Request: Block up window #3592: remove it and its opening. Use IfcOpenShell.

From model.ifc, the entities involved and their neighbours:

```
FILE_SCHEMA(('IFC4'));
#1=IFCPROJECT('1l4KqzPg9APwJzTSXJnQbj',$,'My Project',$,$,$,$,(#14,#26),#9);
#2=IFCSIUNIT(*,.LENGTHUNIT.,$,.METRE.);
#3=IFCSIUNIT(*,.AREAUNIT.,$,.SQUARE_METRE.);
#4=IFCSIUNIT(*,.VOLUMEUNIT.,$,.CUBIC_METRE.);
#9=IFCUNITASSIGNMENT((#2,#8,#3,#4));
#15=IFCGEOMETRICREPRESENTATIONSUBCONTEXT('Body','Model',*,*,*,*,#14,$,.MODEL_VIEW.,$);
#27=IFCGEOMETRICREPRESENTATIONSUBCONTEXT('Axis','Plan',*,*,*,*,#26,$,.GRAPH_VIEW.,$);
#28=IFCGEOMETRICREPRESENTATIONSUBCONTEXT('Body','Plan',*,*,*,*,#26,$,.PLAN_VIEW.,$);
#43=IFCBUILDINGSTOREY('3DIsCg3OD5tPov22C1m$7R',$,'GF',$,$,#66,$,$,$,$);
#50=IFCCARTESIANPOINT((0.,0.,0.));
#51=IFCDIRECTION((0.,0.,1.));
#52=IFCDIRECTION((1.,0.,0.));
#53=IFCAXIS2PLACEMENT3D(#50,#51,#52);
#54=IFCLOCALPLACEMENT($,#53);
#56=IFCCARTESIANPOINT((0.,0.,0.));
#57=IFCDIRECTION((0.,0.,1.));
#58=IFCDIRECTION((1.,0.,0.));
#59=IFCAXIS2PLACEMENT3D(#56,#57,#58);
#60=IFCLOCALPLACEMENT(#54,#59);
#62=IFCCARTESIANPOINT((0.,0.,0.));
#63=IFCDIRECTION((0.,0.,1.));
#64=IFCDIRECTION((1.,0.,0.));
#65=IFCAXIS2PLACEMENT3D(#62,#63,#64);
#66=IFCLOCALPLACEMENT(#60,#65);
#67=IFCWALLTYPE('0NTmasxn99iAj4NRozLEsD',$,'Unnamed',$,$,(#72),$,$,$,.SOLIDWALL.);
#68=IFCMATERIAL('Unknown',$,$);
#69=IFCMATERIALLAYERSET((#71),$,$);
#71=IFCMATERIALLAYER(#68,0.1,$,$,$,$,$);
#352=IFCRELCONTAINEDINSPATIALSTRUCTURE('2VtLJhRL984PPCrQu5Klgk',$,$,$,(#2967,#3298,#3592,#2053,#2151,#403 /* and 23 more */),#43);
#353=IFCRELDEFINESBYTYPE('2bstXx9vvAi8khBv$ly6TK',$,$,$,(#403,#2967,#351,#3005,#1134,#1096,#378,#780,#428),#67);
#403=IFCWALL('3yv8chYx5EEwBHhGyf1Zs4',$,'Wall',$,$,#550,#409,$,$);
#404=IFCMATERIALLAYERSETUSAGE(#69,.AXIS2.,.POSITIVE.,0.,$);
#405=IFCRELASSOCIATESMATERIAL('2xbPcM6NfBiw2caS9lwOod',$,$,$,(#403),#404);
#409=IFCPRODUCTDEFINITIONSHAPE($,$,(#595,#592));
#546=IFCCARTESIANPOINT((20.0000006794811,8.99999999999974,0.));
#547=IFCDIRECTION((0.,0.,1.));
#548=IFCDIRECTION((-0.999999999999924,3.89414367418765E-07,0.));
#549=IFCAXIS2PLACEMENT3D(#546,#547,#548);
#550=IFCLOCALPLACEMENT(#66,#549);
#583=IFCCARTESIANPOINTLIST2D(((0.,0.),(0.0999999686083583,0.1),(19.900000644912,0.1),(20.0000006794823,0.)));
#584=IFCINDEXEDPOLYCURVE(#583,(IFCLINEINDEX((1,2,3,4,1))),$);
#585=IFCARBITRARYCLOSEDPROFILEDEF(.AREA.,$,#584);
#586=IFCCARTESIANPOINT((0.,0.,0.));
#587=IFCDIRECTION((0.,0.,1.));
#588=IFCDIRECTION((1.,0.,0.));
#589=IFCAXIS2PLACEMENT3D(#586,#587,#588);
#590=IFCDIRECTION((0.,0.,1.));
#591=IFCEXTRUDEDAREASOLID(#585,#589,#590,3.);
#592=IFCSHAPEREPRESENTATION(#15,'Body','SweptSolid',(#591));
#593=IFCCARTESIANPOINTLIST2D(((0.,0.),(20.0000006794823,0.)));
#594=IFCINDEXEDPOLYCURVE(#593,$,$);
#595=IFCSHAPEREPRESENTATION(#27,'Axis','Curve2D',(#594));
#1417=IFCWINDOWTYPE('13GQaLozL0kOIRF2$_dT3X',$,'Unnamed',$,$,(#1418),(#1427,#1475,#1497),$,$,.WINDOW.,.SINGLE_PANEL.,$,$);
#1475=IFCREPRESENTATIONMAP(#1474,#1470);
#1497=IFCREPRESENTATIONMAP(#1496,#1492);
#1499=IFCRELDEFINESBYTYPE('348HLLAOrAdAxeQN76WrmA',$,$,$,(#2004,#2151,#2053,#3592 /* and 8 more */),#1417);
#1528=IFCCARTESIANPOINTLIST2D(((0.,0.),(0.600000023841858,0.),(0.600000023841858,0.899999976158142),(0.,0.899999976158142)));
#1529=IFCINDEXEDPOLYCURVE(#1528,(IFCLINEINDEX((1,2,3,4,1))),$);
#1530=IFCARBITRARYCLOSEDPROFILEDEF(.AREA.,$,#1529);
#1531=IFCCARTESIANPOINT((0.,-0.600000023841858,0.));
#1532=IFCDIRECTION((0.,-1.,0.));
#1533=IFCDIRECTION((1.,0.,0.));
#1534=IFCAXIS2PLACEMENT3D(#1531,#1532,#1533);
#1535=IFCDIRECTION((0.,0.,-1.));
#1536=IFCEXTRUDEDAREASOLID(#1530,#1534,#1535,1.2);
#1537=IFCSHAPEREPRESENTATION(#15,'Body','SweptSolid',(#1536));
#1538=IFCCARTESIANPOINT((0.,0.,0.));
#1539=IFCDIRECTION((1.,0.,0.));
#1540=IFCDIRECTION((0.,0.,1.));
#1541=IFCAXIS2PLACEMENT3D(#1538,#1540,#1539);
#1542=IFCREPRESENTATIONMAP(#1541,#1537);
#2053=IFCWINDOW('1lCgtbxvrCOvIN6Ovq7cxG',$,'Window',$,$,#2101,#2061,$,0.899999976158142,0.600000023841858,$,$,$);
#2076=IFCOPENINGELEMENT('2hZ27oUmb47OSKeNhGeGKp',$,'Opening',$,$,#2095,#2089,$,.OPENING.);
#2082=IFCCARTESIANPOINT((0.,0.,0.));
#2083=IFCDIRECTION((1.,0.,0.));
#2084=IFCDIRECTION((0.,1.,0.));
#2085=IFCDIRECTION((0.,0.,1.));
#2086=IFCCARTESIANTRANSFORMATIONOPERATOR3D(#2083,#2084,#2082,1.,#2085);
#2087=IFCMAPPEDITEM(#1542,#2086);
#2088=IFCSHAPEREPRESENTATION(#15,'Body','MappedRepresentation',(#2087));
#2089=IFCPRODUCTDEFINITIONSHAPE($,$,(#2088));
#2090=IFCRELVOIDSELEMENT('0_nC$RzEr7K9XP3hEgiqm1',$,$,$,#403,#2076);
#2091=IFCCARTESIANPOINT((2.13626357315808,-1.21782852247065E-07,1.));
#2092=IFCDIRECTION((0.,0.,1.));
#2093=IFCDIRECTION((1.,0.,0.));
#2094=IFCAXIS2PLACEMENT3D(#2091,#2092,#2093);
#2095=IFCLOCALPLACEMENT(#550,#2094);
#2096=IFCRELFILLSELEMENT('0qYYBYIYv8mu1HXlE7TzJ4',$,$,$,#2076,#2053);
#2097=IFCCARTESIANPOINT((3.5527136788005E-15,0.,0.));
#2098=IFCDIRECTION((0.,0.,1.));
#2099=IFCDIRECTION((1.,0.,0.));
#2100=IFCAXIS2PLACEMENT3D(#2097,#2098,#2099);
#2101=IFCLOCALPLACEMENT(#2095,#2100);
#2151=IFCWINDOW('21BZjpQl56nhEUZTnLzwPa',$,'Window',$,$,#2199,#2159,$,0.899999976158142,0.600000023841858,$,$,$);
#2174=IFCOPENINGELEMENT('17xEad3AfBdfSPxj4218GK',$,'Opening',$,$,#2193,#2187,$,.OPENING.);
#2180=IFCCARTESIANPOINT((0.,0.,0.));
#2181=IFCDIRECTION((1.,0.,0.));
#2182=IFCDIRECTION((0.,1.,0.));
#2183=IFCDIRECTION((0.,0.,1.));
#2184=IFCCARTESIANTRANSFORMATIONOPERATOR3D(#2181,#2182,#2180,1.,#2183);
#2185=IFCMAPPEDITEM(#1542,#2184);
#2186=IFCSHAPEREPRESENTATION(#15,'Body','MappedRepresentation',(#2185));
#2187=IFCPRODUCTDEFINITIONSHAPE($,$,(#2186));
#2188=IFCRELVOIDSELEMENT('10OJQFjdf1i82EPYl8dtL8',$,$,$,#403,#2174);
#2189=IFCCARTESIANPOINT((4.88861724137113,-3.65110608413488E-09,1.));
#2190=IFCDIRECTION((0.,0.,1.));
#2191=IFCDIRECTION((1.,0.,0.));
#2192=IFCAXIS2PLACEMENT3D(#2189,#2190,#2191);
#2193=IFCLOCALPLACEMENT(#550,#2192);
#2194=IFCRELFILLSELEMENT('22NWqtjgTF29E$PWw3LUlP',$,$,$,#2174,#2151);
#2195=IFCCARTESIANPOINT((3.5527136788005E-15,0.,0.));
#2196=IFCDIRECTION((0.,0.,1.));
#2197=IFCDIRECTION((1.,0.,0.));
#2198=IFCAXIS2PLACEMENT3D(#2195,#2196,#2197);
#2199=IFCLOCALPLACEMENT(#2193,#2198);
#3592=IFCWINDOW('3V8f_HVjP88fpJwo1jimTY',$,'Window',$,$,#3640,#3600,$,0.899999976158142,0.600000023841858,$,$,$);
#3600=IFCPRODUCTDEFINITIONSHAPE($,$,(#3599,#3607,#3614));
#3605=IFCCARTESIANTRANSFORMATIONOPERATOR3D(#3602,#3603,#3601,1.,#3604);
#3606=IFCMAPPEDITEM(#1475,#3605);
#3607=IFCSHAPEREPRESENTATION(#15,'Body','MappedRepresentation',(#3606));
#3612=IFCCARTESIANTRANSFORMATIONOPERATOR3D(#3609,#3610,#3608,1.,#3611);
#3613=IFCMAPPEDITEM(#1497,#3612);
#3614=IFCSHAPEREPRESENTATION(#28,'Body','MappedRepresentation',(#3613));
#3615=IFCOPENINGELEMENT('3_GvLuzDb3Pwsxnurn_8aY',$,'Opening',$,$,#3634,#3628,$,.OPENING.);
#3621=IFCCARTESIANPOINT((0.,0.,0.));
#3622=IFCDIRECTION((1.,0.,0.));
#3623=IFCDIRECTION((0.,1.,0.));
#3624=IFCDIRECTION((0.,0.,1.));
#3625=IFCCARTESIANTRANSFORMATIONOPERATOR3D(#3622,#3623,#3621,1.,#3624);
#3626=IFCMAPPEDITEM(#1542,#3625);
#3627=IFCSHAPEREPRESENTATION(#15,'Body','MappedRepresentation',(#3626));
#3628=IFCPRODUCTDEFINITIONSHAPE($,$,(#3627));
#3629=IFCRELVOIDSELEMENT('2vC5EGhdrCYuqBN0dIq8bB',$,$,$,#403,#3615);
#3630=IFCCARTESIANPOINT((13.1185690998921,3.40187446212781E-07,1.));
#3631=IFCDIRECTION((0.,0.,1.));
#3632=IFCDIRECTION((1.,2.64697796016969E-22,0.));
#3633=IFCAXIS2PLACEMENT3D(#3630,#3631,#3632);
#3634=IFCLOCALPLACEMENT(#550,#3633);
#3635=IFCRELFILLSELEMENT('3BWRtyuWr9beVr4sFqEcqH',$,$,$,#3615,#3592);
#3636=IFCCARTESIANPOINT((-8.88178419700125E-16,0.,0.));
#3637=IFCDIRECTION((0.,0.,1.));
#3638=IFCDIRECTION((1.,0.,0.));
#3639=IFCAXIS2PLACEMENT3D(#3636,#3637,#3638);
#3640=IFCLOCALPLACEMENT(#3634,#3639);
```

```python
import ifcopenshell
import ifcopenshell.api.feature
import ifcopenshell.api.root
import ifcopenshell.geom
import ifcopenshell.util.shape

model = ifcopenshell.open("model.ifc")
settings = ifcopenshell.geom.settings()


def volume(element):
    """Net volume in cubic metres, openings subtracted."""
    shape = ifcopenshell.geom.create_shape(settings, element)
    return ifcopenshell.util.shape.get_volume(shape.geometry)


window = model.by_id(3592)
opening = window.FillsVoids[0].RelatingOpeningElement
wall = opening.VoidsElements[0].RelatingBuildingElement
before = volume(wall)

ifcopenshell.api.root.remove_product(model, product=window)
ifcopenshell.api.feature.remove_feature(model, feature=opening)

after = volume(wall)

print(f"wall volume {before:.3f} -> {after:.3f} m3")

model.write("model_updated.ifc")
```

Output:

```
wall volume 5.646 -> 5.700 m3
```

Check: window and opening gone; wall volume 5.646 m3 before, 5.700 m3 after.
